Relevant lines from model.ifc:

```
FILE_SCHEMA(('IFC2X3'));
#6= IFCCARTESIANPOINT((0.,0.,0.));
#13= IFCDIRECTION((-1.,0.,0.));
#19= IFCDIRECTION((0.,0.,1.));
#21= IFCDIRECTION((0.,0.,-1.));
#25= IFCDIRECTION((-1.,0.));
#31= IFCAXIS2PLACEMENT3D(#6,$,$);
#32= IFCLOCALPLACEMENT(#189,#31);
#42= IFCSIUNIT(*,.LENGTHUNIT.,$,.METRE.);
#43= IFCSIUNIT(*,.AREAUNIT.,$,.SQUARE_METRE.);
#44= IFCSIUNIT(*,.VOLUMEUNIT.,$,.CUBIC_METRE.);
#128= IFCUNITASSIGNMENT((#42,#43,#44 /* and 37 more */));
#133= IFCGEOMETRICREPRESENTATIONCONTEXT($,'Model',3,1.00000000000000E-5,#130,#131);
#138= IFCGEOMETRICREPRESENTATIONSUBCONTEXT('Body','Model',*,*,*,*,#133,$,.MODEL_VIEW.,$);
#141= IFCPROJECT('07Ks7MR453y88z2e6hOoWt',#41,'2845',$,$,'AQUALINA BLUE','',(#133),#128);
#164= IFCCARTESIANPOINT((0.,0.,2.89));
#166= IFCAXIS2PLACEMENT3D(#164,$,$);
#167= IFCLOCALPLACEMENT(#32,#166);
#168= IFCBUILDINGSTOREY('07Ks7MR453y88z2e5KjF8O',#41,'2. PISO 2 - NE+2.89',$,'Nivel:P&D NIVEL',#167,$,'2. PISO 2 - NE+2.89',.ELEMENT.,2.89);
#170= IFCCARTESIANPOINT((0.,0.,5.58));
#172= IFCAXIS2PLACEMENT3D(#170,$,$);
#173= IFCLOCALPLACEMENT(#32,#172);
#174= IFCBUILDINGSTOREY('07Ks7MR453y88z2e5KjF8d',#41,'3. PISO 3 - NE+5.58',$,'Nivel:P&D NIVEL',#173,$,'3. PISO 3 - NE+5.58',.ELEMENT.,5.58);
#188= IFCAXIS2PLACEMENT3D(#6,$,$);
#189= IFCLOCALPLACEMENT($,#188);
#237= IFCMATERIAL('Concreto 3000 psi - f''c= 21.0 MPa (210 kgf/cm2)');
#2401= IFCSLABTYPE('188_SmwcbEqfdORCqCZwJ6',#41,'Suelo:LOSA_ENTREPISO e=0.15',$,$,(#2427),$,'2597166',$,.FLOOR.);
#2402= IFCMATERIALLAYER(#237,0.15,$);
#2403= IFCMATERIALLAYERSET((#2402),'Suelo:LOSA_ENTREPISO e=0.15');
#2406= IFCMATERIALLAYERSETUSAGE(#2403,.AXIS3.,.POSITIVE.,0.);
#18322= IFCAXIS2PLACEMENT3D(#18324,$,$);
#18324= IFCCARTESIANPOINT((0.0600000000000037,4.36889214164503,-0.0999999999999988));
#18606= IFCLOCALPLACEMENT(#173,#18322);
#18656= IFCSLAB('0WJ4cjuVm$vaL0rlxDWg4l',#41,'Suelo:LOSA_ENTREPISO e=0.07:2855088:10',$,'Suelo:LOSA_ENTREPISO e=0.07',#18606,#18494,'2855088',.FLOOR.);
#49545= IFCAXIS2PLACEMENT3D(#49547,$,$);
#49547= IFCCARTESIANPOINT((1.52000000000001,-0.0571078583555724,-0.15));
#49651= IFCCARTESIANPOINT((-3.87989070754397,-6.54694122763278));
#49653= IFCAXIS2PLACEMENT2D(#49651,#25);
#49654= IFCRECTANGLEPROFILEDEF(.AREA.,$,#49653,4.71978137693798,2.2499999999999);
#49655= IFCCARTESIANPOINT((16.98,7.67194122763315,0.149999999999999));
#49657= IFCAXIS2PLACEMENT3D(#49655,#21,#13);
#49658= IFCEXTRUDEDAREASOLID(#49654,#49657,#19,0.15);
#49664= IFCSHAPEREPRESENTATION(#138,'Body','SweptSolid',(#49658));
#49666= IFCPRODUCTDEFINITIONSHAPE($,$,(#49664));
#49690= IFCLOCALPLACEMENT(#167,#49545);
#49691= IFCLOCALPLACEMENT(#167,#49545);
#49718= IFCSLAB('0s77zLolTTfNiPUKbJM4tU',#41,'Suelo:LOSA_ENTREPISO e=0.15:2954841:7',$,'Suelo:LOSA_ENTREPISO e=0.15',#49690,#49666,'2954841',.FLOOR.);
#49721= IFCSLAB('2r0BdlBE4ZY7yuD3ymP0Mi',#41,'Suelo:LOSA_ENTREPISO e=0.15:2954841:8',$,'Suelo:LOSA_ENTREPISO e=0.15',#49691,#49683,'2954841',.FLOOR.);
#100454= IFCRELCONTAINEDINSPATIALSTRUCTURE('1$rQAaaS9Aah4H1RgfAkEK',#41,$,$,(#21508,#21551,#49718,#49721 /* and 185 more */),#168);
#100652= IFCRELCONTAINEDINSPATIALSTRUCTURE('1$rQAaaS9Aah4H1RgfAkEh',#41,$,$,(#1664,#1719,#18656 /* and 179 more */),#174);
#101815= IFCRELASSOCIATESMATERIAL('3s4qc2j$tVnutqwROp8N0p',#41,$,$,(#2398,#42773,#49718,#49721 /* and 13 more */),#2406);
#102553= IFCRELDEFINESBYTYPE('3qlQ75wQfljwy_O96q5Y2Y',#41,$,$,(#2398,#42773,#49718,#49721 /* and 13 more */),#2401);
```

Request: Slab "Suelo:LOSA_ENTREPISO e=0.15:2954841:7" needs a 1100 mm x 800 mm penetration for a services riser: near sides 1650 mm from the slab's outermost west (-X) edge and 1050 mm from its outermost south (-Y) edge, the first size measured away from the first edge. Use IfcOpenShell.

```python
import numpy as np
import ifcopenshell
import ifcopenshell.api.feature
import ifcopenshell.api.geometry
import ifcopenshell.api.root
import ifcopenshell.geom
import ifcopenshell.util.placement
import ifcopenshell.util.representation
import ifcopenshell.util.shape
import ifcopenshell.util.unit

model = ifcopenshell.open("model.ifc")
unit_scale = ifcopenshell.util.unit.calculate_unit_scale(model)
settings = ifcopenshell.geom.settings()


def volume(element):
    """Net volume in cubic metres, openings subtracted."""
    shape = ifcopenshell.geom.create_shape(settings, element)
    return ifcopenshell.util.shape.get_volume(shape.geometry)


slab = model.by_guid("0s77zLolTTfNiPUKbJM4tU")
before = volume(slab)

# Extent in the slab's own axes, in metres. The edges named are its -X and -Y sides.
slab_shape = ifcopenshell.geom.create_shape(settings, slab)
vertices = ifcopenshell.util.shape.get_vertices(slab_shape.geometry)
x_min, y_min, bottom = vertices.min(axis=0)
top = vertices[:, 2].max()

opening = ifcopenshell.api.root.create_entity(model, ifc_class="IfcOpeningElement", name="Services riser opening")
context = ifcopenshell.util.representation.get_context(model, "Model", "Body", "MODEL_VIEW")
width, depth = 1.1, 0.8
outline = [(0.0, 0.0), (width, 0.0), (width, depth), (0.0, depth), (0.0, 0.0)]
# Overshoot both faces by 50 mm so the cut is clean.
shape = ifcopenshell.api.geometry.add_slab_representation(
    model, context=context, depth=top - bottom + 0.1, polyline=outline
)
ifcopenshell.api.geometry.assign_representation(model, product=opening, representation=shape)

matrix = ifcopenshell.util.placement.get_local_placement(slab.ObjectPlacement)
matrix[:, 3] = matrix @ np.append(np.array([x_min + 1.65, y_min + 1.05, bottom - 0.05]) / unit_scale, 1.0)
ifcopenshell.api.geometry.edit_object_placement(model, product=opening, matrix=matrix, is_si=False)
ifcopenshell.api.feature.add_feature(model, feature=opening, element=slab)

after = volume(slab)

print(f"slab volume {before:.3f} -> {after:.3f} m3")

model.write("model-out.ifc")
```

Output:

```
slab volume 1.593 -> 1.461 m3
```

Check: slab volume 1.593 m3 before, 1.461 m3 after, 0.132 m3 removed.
